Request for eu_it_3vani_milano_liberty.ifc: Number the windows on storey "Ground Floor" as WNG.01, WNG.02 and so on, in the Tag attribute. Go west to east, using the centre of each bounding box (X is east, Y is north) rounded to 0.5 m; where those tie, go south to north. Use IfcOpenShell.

First a look at what the model holds.

```python
import ifcopenshell
import ifcopenshell.util.element
import ifcopenshell.util.placement

model = ifcopenshell.open("eu_it_3vani_milano_liberty.ifc")
print(model.schema)
storey = next(s for s in model.by_type("IfcBuildingStorey") if s.Name == "Ground Floor")
windows = [e for e in ifcopenshell.util.element.get_decomposition(storey) if e.is_a("IfcWindow")]
for e in sorted(windows, key=lambda e: e.id()):
    origin = ifcopenshell.util.placement.get_local_placement(e.ObjectPlacement)[:3, 3]
    print(e.id(), e.Tag, e.Name, origin.round(2) + 0.0, sep=" | ")
```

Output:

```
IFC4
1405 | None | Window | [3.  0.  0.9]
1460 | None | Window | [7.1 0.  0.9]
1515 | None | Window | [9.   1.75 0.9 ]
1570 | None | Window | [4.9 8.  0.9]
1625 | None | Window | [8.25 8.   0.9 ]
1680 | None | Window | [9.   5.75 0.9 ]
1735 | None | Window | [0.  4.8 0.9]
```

```python
import ifcopenshell
import ifcopenshell.geom
import ifcopenshell.util.element
import ifcopenshell.util.shape

model = ifcopenshell.open("eu_it_3vani_milano_liberty.ifc")
settings = ifcopenshell.geom.settings()
settings.set("use-world-coords", True)


def centre(element):
    shape = ifcopenshell.geom.create_shape(settings, element)
    return ifcopenshell.util.shape.get_bbox_centroid(shape.geometry)


storey = next(s for s in model.by_type("IfcBuildingStorey") if s.Name == "Ground Floor")
windows = [e for e in ifcopenshell.util.element.get_decomposition(storey) if e.is_a("IfcWindow")]

# Insertion points can sit at a corner or the storey origin, so sort by the geometry (in metres).
centres = {e: centre(e) for e in windows}
windows.sort(key=lambda e: (round(centres[e][0] / 0.5), centres[e][1]))

for i, e in enumerate(windows, start=1):
    number = f"WNG.{i:02d}"
    e.Tag = number
    print(e.id(), number)

model.write("eu_it_3vani_milano_liberty_v2.ifc")
```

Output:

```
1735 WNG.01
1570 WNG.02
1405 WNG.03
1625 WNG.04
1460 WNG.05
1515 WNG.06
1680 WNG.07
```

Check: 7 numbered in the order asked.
